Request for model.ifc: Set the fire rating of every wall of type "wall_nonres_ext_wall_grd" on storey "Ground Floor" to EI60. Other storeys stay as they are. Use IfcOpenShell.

First a look at what the model holds.

```python
import ifcopenshell
import ifcopenshell.util.element

model = ifcopenshell.open("model.ifc")
print(model.schema)
storey = next(s for s in model.by_type("IfcBuildingStorey") if s.Name == "Ground Floor")
walls = [e for e in ifcopenshell.util.element.get_decomposition(storey) if e.is_a("IfcWall")]
seen = {}
for e in walls:
    element_type = ifcopenshell.util.element.get_type(e)
    key = (element_type.Name if element_type != e and element_type else None, ifcopenshell.util.element.get_pset(e, "Pset_WallCommon", "FireRating"))
    seen[key] = seen.get(key, 0) + 1
for (name, value), count in sorted(seen.items(), key=str):
    print(count, "x", name, "|", value)
```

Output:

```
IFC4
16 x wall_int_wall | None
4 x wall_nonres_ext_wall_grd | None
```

```python
import ifcopenshell
import ifcopenshell.api.pset
import ifcopenshell.util.element

model = ifcopenshell.open("model.ifc")

storey = next(s for s in model.by_type("IfcBuildingStorey") if s.Name == "Ground Floor")
walls = [e for e in ifcopenshell.util.element.get_decomposition(storey) if e.is_a("IfcWall")]

count = 0
for e in walls:
    element_type = ifcopenshell.util.element.get_type(e)
    if element_type in (None, e) or element_type.Name != "wall_nonres_ext_wall_grd":
        continue
    # add_pset returns the element's existing set when there is one.
    pset = ifcopenshell.api.pset.add_pset(model, product=e, name="Pset_WallCommon")
    ifcopenshell.api.pset.edit_pset(model, pset=pset, properties={"FireRating": "EI60"})
    count += 1

print(count, "walls updated")

model.write("model-out.ifc")
```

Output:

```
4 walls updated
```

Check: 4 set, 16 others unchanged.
